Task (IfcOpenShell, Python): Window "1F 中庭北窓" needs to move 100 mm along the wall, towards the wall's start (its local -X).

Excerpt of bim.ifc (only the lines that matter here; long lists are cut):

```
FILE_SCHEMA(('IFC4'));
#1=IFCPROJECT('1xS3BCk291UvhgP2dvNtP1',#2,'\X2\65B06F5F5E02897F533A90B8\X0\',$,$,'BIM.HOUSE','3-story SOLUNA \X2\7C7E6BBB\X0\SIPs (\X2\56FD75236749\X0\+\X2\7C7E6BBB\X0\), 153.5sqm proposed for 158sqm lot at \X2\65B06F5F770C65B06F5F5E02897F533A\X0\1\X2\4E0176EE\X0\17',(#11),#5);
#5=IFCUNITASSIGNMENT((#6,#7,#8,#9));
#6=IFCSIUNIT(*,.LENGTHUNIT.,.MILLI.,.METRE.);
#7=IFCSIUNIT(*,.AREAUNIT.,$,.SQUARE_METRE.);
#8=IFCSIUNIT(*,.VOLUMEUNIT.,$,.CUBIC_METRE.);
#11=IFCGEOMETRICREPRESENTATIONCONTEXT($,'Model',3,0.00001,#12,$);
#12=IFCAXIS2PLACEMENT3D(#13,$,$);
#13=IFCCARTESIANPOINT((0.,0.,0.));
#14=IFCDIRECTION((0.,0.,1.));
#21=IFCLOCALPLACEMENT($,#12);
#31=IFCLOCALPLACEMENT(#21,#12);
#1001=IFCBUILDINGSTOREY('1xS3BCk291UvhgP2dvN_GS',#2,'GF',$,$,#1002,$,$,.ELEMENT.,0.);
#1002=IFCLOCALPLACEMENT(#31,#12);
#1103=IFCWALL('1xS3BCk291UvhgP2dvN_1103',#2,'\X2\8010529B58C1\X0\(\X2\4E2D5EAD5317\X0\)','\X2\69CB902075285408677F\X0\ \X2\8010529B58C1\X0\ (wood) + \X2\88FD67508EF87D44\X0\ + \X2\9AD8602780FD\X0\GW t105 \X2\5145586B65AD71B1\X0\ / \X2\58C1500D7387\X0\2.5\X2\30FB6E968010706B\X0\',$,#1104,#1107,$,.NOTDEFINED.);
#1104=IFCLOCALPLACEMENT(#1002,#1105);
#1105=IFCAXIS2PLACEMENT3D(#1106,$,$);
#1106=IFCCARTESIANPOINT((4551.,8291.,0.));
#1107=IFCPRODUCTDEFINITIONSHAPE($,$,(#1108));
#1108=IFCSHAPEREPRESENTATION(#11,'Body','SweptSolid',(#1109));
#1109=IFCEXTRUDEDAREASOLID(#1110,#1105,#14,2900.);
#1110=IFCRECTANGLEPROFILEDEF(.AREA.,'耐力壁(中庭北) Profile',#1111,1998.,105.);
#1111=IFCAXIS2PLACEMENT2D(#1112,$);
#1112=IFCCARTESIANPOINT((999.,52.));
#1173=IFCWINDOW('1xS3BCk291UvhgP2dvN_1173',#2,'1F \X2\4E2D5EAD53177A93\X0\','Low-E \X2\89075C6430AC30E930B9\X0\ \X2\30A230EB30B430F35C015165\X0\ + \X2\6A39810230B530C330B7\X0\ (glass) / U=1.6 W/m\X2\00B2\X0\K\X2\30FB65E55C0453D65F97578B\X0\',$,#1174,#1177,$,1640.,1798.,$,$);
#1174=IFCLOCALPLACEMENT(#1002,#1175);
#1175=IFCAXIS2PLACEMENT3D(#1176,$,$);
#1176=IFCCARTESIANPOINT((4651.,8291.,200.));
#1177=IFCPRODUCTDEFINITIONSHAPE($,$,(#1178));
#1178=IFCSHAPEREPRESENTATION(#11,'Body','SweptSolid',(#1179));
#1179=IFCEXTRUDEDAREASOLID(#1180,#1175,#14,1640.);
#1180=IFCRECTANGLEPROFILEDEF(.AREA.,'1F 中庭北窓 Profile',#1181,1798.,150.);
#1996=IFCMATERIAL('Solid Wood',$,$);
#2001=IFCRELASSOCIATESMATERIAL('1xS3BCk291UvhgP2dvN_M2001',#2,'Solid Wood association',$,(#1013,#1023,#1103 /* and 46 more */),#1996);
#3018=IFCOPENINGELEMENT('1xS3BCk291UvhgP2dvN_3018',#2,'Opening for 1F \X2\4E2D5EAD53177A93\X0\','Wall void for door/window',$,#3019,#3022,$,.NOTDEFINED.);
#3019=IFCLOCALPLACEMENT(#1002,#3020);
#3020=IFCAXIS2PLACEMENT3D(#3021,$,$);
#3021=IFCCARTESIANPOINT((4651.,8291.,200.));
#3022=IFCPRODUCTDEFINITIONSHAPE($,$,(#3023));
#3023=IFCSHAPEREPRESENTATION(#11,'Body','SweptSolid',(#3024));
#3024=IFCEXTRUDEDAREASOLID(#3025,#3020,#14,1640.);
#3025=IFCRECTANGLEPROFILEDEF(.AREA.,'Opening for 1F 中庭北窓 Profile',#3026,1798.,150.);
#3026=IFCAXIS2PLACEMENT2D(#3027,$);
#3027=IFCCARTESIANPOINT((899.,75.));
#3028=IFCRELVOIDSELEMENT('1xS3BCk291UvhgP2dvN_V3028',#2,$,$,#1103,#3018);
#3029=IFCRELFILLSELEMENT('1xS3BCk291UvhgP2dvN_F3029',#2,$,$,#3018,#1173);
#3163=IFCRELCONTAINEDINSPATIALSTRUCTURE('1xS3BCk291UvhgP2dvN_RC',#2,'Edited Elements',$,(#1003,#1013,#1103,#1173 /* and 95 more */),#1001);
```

```python
import ifcopenshell
import ifcopenshell.api.geometry
import ifcopenshell.util.placement
import ifcopenshell.util.unit

model = ifcopenshell.open("bim.ifc")
unit_scale = ifcopenshell.util.unit.calculate_unit_scale(model)

window = model.by_guid("1xS3BCk291UvhgP2dvN_1173")
opening = window.FillsVoids[0].RelatingOpeningElement
wall = opening.VoidsElements[0].RelatingBuildingElement

wall_matrix = ifcopenshell.util.placement.get_local_placement(wall.ObjectPlacement)
shift = wall_matrix[:3, 0] * -0.1 / unit_scale
before = ifcopenshell.util.placement.get_local_placement(window.ObjectPlacement)[:3, 3].copy()

# The window is not placed relative to its opening, so move both.
for product in (opening, window):
    matrix = ifcopenshell.util.placement.get_local_placement(product.ObjectPlacement)
    matrix[:3, 3] += shift
    ifcopenshell.api.geometry.edit_object_placement(model, product=product, matrix=matrix, is_si=False)

after = ifcopenshell.util.placement.get_local_placement(window.ObjectPlacement)[:3, 3]
print("window moved by", (after - before).round(3) + 0.0)

model.write("bim_v2.ifc")
```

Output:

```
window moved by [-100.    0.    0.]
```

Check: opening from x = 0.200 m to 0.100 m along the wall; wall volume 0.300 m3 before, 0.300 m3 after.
